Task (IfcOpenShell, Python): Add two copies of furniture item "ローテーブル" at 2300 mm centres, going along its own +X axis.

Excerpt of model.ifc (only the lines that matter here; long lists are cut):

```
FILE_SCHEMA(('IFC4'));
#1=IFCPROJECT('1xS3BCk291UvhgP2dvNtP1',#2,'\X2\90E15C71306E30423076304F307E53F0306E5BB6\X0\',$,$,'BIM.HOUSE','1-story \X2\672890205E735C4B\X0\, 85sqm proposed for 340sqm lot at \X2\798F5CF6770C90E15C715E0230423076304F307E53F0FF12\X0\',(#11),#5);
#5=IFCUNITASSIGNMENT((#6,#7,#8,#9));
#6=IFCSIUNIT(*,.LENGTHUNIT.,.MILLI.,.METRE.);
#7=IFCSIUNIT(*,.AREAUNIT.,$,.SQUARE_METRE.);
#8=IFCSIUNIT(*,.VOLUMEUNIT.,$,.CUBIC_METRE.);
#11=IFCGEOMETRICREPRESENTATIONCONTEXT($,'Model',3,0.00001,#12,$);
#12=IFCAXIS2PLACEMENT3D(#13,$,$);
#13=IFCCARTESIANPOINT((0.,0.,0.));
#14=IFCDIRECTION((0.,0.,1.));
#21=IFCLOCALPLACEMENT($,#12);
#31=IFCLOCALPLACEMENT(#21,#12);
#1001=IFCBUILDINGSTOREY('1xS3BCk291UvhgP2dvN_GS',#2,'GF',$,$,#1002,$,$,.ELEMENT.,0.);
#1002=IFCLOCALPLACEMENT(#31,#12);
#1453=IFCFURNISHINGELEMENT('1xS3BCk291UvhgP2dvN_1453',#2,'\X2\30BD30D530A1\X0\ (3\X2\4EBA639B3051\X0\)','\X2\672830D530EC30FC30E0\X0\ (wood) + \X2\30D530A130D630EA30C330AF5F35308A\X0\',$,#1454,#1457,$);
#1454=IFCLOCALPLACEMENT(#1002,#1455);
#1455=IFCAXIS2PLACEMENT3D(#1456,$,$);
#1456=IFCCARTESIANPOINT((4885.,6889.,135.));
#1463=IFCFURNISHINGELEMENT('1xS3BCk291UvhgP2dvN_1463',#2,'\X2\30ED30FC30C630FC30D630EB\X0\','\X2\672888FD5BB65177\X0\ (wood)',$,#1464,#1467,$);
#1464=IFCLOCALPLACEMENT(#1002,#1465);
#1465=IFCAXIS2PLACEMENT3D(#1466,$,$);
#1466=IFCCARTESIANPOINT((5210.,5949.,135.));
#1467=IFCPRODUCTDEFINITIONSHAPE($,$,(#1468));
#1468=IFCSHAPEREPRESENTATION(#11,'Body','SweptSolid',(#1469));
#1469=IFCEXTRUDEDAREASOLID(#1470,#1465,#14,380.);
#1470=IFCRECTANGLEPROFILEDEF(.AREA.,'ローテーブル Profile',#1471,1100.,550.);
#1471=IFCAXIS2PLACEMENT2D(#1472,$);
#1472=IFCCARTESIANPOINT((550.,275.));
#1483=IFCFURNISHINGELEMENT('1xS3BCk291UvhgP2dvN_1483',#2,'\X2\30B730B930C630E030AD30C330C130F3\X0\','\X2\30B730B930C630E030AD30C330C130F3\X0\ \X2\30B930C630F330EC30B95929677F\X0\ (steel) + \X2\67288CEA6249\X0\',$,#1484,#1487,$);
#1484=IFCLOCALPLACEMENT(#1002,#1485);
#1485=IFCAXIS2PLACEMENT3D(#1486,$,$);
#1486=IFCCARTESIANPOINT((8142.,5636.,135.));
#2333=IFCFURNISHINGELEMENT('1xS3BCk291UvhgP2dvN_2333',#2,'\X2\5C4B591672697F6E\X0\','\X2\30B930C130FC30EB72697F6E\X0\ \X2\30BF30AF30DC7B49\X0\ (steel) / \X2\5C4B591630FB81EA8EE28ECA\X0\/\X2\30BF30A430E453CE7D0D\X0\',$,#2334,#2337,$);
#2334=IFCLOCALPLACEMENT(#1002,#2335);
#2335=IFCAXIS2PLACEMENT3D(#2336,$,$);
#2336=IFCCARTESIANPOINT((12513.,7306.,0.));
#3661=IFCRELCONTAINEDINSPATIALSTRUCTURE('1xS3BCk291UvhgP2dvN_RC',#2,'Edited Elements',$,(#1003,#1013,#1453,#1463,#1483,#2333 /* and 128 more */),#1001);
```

```python
import ifcopenshell
import ifcopenshell.api.geometry
import ifcopenshell.api.root
import ifcopenshell.util.element
import ifcopenshell.util.placement
import ifcopenshell.util.unit

model = ifcopenshell.open("model.ifc")
unit_scale = ifcopenshell.util.unit.calculate_unit_scale(model)


def reuse_history(source, copy):
    """copy_class also copies each property set's owner history, people and application; keep the originals."""
    for rel in copy.IsDefinedBy:
        if rel.is_a("IfcRelDefinesByProperties") and (history := rel.RelatingPropertyDefinition.OwnerHistory):
            rel.RelatingPropertyDefinition.OwnerHistory = source.OwnerHistory
            ifcopenshell.util.element.remove_deep2(model, history)


source = model.by_id(1463)
base = ifcopenshell.util.placement.get_local_placement(source.ObjectPlacement)
step = base[:3, 0] * 2.3 / unit_scale

for i in range(1, 3):
    copy = ifcopenshell.api.root.copy_class(model, product=source)
    copy.Representation = ifcopenshell.util.element.copy_deep(
        model, source.Representation, exclude=["IfcGeometricRepresentationContext", "IfcRepresentationMap"]
    )
    reuse_history(source, copy)
    matrix = base.copy()
    matrix[:3, 3] += i * step
    print("added at", matrix[:3, 3].round(3) + 0.0)
    ifcopenshell.api.geometry.edit_object_placement(model, product=copy, matrix=matrix, is_si=False)

model.write("model_updated.ifc")
```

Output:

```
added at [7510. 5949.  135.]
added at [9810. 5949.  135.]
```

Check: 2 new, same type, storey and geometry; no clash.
